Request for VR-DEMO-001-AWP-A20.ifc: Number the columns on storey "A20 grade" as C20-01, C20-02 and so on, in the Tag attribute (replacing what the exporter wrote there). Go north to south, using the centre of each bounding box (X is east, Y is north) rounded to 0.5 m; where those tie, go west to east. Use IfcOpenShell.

First a look at what the model holds.

```python
import ifcopenshell
import ifcopenshell.util.element
import ifcopenshell.util.placement

model = ifcopenshell.open("VR-DEMO-001-AWP-A20.ifc")
print(model.schema)
storey = next(s for s in model.by_type("IfcBuildingStorey") if s.Name == "A20 grade")
columns = [e for e in ifcopenshell.util.element.get_decomposition(storey) if e.is_a("IfcColumn")]
for e in sorted(columns, key=lambda e: e.id()):
    origin = ifcopenshell.util.placement.get_local_placement(e.ObjectPlacement)[:3, 3]
    print(e.id(), e.Tag, e.Name, origin.round(2) + 0.0, sep=" | ")
```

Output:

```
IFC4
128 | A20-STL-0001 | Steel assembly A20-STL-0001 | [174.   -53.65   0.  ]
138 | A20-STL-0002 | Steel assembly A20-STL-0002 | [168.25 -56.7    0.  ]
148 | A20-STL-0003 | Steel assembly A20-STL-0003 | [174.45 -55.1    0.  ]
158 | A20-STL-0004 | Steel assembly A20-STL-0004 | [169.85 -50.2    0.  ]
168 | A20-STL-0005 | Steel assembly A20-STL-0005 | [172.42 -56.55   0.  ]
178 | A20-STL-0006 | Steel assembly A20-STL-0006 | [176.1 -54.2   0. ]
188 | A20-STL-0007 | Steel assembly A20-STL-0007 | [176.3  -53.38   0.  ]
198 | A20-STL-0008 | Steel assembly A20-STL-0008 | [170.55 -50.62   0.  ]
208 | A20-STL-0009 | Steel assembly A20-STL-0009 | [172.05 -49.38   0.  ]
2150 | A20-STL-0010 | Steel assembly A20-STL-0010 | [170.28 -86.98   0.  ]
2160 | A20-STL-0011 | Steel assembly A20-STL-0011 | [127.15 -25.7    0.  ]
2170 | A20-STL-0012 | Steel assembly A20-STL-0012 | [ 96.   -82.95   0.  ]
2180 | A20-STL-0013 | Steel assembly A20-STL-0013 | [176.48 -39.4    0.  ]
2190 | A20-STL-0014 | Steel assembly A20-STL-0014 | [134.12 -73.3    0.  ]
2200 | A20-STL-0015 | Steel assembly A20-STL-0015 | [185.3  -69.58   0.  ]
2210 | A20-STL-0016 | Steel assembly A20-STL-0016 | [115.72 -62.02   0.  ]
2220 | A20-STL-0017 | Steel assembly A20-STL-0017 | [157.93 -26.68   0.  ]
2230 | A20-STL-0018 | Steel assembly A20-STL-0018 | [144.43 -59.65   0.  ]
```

```python
import ifcopenshell
import ifcopenshell.geom
import ifcopenshell.util.element
import ifcopenshell.util.shape

model = ifcopenshell.open("VR-DEMO-001-AWP-A20.ifc")
settings = ifcopenshell.geom.settings()
settings.set("use-world-coords", True)


def centre(element):
    shape = ifcopenshell.geom.create_shape(settings, element)
    return ifcopenshell.util.shape.get_bbox_centroid(shape.geometry)


storey = next(s for s in model.by_type("IfcBuildingStorey") if s.Name == "A20 grade")
columns = [e for e in ifcopenshell.util.element.get_decomposition(storey) if e.is_a("IfcColumn")]

# Insertion points can sit at a corner or the storey origin, so sort by the geometry (in metres).
centres = {e: centre(e) for e in columns}
columns.sort(key=lambda e: (-round(centres[e][1] / 0.5), centres[e][0]))

for i, e in enumerate(columns, start=1):
    number = f"C20-{i:02d}"
    e.Tag = number
    print(e.id(), number)

model.write("VR-DEMO-001-AWP-A20-out.ifc")
```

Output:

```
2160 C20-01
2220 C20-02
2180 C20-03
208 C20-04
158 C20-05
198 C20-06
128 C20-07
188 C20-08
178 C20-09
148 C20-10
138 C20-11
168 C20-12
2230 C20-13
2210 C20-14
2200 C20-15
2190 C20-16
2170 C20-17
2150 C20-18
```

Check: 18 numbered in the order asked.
